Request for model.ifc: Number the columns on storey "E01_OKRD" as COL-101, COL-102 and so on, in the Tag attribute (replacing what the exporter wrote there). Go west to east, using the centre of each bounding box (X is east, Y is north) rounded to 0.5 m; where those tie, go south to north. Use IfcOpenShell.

First a look at what the model holds.

```python
import ifcopenshell
import ifcopenshell.util.element
import ifcopenshell.util.placement

model = ifcopenshell.open("model.ifc")
print(model.schema)
storey = next(s for s in model.by_type("IfcBuildingStorey") if s.Name == "E01_OKRD")
columns = [e for e in ifcopenshell.util.element.get_decomposition(storey) if e.is_a("IfcColumn")]
for e in sorted(columns, key=lambda e: e.id()):
    origin = ifcopenshell.util.placement.get_local_placement(e.ObjectPlacement)[:3, 3]
    print(e.id(), e.Tag, e.Name, origin.round(2) + 0.0, sep=" | ")
```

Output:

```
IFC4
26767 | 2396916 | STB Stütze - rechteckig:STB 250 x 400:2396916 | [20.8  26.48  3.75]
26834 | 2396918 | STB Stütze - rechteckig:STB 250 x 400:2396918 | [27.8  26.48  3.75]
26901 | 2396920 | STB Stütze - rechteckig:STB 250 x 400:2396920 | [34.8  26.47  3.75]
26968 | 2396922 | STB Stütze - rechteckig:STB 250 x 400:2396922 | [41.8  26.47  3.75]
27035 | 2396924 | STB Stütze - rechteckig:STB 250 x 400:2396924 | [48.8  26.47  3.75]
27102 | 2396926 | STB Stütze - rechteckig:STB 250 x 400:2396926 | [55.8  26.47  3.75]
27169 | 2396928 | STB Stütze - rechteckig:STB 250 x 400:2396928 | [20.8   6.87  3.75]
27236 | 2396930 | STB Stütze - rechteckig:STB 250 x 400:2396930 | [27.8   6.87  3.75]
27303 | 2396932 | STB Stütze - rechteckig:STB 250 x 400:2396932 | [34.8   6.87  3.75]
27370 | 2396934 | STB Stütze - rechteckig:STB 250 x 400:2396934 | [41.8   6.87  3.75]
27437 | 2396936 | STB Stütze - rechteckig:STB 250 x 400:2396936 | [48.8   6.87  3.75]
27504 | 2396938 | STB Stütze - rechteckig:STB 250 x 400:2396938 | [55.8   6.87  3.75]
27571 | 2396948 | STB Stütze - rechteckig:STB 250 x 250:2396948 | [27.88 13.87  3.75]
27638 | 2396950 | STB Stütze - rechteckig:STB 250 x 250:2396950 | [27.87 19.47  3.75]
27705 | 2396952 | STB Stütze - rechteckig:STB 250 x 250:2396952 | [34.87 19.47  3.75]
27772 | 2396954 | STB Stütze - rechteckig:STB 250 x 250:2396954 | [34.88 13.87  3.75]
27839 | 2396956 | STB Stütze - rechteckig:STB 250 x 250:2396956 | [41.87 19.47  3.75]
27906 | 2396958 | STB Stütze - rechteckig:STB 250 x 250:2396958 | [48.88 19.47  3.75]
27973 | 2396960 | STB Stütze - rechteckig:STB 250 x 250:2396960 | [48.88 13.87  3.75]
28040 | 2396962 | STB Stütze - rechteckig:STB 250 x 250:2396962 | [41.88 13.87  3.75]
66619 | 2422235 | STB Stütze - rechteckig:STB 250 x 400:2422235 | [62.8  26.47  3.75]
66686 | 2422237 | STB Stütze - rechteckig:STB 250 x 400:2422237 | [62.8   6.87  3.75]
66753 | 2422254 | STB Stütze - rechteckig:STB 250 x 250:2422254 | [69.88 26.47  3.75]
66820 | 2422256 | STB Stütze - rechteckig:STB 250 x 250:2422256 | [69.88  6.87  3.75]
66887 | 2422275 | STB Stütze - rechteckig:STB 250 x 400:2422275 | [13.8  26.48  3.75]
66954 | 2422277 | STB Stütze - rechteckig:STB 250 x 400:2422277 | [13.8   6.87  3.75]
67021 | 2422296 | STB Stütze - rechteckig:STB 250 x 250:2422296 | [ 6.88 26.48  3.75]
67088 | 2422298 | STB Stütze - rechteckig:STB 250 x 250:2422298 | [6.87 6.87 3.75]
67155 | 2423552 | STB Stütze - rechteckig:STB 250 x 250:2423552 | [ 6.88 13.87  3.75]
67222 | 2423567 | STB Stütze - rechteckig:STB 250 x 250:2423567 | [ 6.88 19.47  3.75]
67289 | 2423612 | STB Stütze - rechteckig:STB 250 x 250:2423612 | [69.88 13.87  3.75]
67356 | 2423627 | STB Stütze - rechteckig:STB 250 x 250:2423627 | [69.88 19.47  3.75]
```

```python
import ifcopenshell
import ifcopenshell.geom
import ifcopenshell.util.element
import ifcopenshell.util.shape

model = ifcopenshell.open("model.ifc")
settings = ifcopenshell.geom.settings()
settings.set("use-world-coords", True)


def centre(element):
    shape = ifcopenshell.geom.create_shape(settings, element)
    return ifcopenshell.util.shape.get_bbox_centroid(shape.geometry)


storey = next(s for s in model.by_type("IfcBuildingStorey") if s.Name == "E01_OKRD")
columns = [e for e in ifcopenshell.util.element.get_decomposition(storey) if e.is_a("IfcColumn")]

# Insertion points can sit at a corner or the storey origin, so sort by the geometry (in metres).
centres = {e: centre(e) for e in columns}
columns.sort(key=lambda e: (round(centres[e][0] / 0.5), centres[e][1]))

for i, e in enumerate(columns, start=1):
    number = f"COL-1{i:02d}"
    e.Tag = number
    print(e.id(), number)

model.write("model_v2.ifc")
```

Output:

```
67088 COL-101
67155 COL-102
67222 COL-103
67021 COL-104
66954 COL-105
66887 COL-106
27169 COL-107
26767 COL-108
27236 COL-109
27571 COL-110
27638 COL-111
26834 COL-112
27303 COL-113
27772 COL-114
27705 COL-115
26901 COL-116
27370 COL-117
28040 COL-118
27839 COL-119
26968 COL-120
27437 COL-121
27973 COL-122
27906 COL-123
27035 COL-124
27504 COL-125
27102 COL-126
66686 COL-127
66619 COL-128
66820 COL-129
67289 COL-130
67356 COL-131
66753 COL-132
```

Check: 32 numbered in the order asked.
